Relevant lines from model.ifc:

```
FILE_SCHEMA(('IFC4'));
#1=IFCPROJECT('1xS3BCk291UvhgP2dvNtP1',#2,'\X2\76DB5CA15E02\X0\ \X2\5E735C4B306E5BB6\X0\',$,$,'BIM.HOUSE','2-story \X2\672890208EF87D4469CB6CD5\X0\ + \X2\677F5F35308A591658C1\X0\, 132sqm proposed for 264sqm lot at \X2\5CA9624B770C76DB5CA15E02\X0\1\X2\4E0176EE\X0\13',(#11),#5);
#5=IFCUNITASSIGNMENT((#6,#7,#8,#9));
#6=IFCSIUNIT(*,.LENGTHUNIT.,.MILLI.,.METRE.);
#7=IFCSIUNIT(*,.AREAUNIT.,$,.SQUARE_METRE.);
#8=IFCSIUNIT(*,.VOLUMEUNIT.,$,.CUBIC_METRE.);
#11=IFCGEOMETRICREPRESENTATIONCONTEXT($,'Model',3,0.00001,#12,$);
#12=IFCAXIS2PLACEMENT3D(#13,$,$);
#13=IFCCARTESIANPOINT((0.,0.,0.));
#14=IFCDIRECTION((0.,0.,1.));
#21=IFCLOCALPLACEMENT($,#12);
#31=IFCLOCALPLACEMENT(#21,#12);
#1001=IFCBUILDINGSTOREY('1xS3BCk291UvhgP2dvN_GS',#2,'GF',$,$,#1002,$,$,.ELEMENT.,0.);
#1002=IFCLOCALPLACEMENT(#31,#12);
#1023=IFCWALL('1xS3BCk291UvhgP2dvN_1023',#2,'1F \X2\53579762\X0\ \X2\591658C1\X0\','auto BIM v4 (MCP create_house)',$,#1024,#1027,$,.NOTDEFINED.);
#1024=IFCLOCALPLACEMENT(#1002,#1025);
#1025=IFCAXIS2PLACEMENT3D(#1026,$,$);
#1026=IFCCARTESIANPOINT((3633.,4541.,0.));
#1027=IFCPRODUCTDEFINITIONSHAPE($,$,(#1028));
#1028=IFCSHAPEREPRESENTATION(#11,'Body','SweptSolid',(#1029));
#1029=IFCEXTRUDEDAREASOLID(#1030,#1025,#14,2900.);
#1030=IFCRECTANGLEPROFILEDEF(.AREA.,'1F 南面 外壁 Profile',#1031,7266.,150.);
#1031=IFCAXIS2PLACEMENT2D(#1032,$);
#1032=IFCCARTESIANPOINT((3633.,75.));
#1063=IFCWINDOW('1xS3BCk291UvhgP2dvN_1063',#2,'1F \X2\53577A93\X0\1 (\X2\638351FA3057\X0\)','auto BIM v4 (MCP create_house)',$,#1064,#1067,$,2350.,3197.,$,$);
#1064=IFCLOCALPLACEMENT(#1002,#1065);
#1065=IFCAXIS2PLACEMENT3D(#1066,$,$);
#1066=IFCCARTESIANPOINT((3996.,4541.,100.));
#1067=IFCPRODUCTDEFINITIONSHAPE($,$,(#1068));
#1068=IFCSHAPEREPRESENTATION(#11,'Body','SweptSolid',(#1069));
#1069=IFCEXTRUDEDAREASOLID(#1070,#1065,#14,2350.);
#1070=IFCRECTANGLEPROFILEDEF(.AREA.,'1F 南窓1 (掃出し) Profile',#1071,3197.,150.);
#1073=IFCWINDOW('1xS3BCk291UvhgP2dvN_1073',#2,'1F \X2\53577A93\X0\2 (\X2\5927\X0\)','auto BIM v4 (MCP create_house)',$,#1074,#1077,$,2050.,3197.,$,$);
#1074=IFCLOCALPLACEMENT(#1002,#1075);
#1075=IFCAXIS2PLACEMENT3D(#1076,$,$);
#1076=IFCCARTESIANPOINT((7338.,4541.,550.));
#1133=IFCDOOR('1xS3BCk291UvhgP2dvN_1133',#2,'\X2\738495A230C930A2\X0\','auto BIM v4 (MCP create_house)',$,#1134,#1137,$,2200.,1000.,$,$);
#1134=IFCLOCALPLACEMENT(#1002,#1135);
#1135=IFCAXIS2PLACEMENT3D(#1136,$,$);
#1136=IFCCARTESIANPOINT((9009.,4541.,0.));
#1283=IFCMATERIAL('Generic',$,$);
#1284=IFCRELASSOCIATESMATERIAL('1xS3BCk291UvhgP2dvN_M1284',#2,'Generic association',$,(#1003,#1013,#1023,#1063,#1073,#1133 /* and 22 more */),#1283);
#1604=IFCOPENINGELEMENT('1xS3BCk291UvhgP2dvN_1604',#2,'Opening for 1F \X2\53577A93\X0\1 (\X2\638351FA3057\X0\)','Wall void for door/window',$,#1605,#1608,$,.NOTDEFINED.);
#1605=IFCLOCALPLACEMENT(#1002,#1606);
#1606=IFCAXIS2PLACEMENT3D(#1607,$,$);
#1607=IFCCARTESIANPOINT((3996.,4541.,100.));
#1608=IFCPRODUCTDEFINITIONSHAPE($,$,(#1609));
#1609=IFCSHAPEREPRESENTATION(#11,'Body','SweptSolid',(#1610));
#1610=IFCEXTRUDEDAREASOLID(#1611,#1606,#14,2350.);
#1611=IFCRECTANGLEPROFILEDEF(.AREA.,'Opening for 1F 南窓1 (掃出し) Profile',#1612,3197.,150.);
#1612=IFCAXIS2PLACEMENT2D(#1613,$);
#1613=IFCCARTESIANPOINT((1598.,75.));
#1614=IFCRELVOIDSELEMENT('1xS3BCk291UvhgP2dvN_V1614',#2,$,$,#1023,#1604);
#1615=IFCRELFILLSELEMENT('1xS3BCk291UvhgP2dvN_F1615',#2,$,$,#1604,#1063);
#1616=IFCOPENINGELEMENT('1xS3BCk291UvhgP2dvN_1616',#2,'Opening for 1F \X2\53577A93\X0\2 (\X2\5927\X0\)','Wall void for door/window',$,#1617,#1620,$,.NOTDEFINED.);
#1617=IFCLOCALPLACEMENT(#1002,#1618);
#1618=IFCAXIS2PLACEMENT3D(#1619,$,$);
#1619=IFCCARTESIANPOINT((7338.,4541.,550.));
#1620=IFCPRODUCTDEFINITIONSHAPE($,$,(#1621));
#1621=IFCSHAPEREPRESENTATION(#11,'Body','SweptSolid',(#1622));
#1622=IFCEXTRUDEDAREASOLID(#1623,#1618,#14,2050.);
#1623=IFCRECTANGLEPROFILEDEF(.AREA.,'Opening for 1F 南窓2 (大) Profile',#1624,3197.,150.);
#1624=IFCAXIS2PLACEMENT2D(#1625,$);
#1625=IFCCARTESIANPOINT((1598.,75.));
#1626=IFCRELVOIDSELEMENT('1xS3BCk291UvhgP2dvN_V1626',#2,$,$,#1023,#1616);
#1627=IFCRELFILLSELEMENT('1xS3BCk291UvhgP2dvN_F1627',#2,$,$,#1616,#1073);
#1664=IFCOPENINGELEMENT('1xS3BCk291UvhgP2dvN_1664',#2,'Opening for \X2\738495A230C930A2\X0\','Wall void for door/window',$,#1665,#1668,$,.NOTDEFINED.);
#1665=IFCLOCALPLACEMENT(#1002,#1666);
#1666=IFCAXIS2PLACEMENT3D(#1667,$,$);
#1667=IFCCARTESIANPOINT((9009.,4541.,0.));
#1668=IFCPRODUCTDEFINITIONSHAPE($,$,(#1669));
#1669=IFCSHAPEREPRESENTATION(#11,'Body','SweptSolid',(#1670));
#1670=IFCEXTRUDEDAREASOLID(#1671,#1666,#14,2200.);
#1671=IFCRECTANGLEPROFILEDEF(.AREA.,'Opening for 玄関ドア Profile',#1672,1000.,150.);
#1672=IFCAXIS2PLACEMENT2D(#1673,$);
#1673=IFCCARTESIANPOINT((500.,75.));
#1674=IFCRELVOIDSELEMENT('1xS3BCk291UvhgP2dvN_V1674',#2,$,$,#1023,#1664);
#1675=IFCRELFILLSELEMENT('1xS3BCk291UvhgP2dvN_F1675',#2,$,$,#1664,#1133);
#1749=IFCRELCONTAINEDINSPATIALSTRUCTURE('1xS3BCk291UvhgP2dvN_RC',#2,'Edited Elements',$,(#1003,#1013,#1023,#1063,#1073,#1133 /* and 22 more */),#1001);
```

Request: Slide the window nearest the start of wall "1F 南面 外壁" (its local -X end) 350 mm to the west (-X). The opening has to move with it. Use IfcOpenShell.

```python
import ifcopenshell
import ifcopenshell.api.geometry
import ifcopenshell.util.placement
import ifcopenshell.util.unit

model = ifcopenshell.open("model.ifc")
unit_scale = ifcopenshell.util.unit.calculate_unit_scale(model)

window = model.by_guid("1xS3BCk291UvhgP2dvN_1063")
opening = window.FillsVoids[0].RelatingOpeningElement
wall = opening.VoidsElements[0].RelatingBuildingElement

wall_matrix = ifcopenshell.util.placement.get_local_placement(wall.ObjectPlacement)
shift = wall_matrix[:3, 0] * -0.35 / unit_scale
before = ifcopenshell.util.placement.get_local_placement(window.ObjectPlacement)[:3, 3].copy()

# The window is not placed relative to its opening, so move both.
for product in (opening, window):
    matrix = ifcopenshell.util.placement.get_local_placement(product.ObjectPlacement)
    matrix[:3, 3] += shift
    ifcopenshell.api.geometry.edit_object_placement(model, product=product, matrix=matrix, is_si=False)

after = ifcopenshell.util.placement.get_local_placement(window.ObjectPlacement)[:3, 3]
print("window moved by", (after - before).round(3) + 0.0)

model.write("model_v2.ifc")
```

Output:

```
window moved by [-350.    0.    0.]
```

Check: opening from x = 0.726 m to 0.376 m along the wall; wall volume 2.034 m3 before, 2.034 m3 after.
